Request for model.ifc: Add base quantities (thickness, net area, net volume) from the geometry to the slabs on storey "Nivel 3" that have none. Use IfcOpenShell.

First a look at what the model holds.

```python
import ifcopenshell
import ifcopenshell.util.element
import ifcopenshell.util.unit

model = ifcopenshell.open("model.ifc")
print(model.schema)
for unit_type in ("LENGTHUNIT", "AREAUNIT", "VOLUMEUNIT"):
    print(unit_type, ifcopenshell.util.unit.calculate_unit_scale(model, unit_type))
storey = next(s for s in model.by_type("IfcBuildingStorey") if s.Name == "Nivel 3")
slabs = [e for e in ifcopenshell.util.element.get_decomposition(storey) if e.is_a("IfcSlab")]
for e in sorted(slabs, key=lambda e: e.id()):
    print(e.id(), e.is_a(), e.Name, list(ifcopenshell.util.element.get_psets(e, qtos_only=True)), sep=" | ")
```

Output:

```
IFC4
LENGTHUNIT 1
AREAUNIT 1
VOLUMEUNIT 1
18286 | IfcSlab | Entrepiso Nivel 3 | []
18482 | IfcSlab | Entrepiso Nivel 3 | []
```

```python
import ifcopenshell
import ifcopenshell.api.pset
import ifcopenshell.geom
import ifcopenshell.util.element
import ifcopenshell.util.shape
import ifcopenshell.util.unit

model = ifcopenshell.open("model.ifc")
unit_scale = ifcopenshell.util.unit.calculate_unit_scale(model)
area_scale = ifcopenshell.util.unit.calculate_unit_scale(model, "AREAUNIT")
volume_scale = ifcopenshell.util.unit.calculate_unit_scale(model, "VOLUMEUNIT")
settings = ifcopenshell.geom.settings()

storey = next(s for s in model.by_type("IfcBuildingStorey") if s.Name == "Nivel 3")
slabs = [e for e in ifcopenshell.util.element.get_decomposition(storey) if e.is_a("IfcSlab")]

for e in sorted(slabs, key=lambda e: e.id()):
    if ifcopenshell.util.element.get_psets(e, qtos_only=True, should_inherit=False):
        continue
    # Geometry comes back in metres, in the element's own axes.
    shape = ifcopenshell.geom.create_shape(settings, e)
    values = {
        "Width": ifcopenshell.util.shape.get_z(shape.geometry) / unit_scale,
        "NetArea": ifcopenshell.util.shape.get_footprint_area(shape.geometry) / area_scale,
        "NetVolume": ifcopenshell.util.shape.get_volume(shape.geometry) / volume_scale,
    }
    qto = ifcopenshell.api.pset.add_qto(model, product=e, name="Qto_SlabBaseQuantities")
    ifcopenshell.api.pset.edit_qto(model, qto=qto, properties=values)
    print(e.id(), {k: round(v, 3) for k, v in values.items()})

model.write("model_rev.ifc")
```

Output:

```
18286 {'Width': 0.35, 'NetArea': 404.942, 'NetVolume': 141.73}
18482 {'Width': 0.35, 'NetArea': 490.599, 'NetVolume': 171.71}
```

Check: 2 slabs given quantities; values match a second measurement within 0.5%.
